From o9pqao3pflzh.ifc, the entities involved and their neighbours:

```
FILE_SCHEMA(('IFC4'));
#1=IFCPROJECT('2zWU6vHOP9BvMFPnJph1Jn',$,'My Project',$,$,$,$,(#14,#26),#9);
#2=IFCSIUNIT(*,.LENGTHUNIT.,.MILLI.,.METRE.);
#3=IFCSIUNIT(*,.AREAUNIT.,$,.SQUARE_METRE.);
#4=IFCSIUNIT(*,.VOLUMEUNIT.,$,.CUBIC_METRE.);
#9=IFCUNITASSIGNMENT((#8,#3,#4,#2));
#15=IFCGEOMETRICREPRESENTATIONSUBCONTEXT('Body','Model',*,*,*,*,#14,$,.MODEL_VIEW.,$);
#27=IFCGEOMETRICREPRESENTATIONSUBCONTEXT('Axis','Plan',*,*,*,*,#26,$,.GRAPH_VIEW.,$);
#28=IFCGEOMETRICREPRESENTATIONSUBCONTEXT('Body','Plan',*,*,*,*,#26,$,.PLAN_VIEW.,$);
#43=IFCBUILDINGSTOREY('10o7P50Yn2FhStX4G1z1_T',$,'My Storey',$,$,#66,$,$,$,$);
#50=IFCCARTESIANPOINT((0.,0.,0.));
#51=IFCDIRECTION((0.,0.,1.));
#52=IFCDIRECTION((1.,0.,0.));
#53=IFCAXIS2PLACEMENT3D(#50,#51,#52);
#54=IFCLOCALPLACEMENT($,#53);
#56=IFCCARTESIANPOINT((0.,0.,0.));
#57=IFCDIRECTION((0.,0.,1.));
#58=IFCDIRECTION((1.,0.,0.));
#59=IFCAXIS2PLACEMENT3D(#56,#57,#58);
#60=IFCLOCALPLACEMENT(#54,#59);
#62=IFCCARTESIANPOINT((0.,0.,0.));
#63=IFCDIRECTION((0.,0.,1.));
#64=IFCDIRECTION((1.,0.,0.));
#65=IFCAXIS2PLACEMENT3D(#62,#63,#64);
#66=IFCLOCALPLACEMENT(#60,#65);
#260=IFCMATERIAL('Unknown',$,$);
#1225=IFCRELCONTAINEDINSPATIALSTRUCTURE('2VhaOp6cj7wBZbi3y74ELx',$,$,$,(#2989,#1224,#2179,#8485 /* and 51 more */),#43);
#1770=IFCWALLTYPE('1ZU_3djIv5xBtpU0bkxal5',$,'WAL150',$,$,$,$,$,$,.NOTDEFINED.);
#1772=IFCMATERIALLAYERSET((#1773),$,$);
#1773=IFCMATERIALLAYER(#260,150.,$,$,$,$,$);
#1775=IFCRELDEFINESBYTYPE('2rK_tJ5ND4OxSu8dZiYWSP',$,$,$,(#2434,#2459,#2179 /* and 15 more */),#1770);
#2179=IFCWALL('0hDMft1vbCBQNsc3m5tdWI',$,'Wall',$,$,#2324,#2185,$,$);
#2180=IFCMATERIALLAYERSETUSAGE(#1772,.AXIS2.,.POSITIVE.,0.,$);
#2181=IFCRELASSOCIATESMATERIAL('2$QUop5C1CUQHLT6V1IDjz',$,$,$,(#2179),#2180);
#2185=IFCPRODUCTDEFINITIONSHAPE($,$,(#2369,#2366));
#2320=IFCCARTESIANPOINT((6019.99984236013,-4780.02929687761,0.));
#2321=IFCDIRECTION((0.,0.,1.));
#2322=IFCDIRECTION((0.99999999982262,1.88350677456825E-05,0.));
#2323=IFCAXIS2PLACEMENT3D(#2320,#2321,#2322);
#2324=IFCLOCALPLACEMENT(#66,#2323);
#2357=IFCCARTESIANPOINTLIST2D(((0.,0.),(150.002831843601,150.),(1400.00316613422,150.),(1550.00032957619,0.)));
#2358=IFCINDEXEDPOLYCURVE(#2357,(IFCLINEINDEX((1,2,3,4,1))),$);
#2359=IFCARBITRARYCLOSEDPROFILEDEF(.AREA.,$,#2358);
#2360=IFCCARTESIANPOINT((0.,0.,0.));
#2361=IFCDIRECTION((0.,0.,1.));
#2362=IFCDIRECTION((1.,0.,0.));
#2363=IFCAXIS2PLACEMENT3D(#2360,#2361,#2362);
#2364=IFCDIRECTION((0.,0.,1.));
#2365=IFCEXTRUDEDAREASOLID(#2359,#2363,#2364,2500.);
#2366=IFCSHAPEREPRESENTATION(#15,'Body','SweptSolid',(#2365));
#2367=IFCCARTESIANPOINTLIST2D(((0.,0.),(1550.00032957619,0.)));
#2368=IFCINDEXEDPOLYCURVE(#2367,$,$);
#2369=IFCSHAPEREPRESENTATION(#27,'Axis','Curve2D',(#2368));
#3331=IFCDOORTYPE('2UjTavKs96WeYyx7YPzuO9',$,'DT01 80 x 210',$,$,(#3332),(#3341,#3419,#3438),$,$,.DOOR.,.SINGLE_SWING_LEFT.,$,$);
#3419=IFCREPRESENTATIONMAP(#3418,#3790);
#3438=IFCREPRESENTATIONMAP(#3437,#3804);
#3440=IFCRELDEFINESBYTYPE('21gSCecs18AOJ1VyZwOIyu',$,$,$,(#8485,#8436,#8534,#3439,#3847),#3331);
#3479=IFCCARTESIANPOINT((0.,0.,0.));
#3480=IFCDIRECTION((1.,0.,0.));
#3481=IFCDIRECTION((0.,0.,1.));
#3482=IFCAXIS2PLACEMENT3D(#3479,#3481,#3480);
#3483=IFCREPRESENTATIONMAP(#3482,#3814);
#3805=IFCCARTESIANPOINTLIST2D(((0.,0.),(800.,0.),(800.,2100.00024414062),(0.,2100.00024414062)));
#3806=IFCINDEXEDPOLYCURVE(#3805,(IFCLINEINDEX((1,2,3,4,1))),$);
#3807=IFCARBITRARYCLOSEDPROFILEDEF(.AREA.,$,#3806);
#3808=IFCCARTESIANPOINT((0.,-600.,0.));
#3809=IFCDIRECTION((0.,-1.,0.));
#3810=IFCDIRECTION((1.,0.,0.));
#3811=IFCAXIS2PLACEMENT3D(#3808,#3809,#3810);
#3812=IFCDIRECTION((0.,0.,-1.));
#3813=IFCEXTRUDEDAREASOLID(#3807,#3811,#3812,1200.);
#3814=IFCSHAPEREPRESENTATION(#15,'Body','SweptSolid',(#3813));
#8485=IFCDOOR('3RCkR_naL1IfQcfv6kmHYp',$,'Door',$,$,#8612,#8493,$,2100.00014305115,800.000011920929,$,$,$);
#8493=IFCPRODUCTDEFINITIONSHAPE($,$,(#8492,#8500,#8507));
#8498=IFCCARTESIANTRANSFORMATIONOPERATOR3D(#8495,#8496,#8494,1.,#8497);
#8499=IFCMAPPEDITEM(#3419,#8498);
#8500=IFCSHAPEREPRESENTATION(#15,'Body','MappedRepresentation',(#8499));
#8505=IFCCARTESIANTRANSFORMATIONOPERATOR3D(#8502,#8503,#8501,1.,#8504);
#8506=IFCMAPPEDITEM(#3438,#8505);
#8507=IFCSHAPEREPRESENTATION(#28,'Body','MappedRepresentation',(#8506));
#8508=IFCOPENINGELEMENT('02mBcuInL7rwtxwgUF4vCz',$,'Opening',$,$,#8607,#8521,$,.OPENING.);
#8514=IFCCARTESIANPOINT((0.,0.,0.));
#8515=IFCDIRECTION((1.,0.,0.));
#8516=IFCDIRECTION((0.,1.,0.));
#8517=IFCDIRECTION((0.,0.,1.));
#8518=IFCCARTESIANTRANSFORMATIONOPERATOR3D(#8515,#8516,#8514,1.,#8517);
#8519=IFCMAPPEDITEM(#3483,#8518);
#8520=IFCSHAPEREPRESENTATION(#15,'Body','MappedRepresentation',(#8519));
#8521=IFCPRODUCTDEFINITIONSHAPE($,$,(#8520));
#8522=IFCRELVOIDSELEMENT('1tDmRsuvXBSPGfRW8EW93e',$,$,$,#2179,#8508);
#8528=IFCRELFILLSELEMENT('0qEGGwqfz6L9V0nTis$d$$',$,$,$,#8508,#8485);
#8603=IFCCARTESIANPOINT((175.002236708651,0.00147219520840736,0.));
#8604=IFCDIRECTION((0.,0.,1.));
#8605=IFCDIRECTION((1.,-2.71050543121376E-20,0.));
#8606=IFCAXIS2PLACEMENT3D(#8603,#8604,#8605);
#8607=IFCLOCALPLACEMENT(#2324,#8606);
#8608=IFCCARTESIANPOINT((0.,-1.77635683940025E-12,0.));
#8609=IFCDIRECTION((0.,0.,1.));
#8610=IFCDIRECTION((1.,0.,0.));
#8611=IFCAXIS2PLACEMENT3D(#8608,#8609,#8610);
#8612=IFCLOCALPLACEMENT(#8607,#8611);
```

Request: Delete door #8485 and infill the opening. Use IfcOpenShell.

```python
import ifcopenshell
import ifcopenshell.api.feature
import ifcopenshell.api.root
import ifcopenshell.geom
import ifcopenshell.util.shape

model = ifcopenshell.open("o9pqao3pflzh.ifc")
settings = ifcopenshell.geom.settings()


def volume(element):
    """Net volume in cubic metres, openings subtracted."""
    shape = ifcopenshell.geom.create_shape(settings, element)
    return ifcopenshell.util.shape.get_volume(shape.geometry)


door = model.by_guid("3RCkR_naL1IfQcfv6kmHYp")
opening = door.FillsVoids[0].RelatingOpeningElement
wall = opening.VoidsElements[0].RelatingBuildingElement
before = volume(wall)

ifcopenshell.api.root.remove_product(model, product=door)
ifcopenshell.api.feature.remove_feature(model, feature=opening)

after = volume(wall)

print(f"wall volume {before:.3f} -> {after:.3f} m3")

model.write("o9pqao3pflzh_v2.ifc")
```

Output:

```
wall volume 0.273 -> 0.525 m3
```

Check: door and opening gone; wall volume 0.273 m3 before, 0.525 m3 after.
